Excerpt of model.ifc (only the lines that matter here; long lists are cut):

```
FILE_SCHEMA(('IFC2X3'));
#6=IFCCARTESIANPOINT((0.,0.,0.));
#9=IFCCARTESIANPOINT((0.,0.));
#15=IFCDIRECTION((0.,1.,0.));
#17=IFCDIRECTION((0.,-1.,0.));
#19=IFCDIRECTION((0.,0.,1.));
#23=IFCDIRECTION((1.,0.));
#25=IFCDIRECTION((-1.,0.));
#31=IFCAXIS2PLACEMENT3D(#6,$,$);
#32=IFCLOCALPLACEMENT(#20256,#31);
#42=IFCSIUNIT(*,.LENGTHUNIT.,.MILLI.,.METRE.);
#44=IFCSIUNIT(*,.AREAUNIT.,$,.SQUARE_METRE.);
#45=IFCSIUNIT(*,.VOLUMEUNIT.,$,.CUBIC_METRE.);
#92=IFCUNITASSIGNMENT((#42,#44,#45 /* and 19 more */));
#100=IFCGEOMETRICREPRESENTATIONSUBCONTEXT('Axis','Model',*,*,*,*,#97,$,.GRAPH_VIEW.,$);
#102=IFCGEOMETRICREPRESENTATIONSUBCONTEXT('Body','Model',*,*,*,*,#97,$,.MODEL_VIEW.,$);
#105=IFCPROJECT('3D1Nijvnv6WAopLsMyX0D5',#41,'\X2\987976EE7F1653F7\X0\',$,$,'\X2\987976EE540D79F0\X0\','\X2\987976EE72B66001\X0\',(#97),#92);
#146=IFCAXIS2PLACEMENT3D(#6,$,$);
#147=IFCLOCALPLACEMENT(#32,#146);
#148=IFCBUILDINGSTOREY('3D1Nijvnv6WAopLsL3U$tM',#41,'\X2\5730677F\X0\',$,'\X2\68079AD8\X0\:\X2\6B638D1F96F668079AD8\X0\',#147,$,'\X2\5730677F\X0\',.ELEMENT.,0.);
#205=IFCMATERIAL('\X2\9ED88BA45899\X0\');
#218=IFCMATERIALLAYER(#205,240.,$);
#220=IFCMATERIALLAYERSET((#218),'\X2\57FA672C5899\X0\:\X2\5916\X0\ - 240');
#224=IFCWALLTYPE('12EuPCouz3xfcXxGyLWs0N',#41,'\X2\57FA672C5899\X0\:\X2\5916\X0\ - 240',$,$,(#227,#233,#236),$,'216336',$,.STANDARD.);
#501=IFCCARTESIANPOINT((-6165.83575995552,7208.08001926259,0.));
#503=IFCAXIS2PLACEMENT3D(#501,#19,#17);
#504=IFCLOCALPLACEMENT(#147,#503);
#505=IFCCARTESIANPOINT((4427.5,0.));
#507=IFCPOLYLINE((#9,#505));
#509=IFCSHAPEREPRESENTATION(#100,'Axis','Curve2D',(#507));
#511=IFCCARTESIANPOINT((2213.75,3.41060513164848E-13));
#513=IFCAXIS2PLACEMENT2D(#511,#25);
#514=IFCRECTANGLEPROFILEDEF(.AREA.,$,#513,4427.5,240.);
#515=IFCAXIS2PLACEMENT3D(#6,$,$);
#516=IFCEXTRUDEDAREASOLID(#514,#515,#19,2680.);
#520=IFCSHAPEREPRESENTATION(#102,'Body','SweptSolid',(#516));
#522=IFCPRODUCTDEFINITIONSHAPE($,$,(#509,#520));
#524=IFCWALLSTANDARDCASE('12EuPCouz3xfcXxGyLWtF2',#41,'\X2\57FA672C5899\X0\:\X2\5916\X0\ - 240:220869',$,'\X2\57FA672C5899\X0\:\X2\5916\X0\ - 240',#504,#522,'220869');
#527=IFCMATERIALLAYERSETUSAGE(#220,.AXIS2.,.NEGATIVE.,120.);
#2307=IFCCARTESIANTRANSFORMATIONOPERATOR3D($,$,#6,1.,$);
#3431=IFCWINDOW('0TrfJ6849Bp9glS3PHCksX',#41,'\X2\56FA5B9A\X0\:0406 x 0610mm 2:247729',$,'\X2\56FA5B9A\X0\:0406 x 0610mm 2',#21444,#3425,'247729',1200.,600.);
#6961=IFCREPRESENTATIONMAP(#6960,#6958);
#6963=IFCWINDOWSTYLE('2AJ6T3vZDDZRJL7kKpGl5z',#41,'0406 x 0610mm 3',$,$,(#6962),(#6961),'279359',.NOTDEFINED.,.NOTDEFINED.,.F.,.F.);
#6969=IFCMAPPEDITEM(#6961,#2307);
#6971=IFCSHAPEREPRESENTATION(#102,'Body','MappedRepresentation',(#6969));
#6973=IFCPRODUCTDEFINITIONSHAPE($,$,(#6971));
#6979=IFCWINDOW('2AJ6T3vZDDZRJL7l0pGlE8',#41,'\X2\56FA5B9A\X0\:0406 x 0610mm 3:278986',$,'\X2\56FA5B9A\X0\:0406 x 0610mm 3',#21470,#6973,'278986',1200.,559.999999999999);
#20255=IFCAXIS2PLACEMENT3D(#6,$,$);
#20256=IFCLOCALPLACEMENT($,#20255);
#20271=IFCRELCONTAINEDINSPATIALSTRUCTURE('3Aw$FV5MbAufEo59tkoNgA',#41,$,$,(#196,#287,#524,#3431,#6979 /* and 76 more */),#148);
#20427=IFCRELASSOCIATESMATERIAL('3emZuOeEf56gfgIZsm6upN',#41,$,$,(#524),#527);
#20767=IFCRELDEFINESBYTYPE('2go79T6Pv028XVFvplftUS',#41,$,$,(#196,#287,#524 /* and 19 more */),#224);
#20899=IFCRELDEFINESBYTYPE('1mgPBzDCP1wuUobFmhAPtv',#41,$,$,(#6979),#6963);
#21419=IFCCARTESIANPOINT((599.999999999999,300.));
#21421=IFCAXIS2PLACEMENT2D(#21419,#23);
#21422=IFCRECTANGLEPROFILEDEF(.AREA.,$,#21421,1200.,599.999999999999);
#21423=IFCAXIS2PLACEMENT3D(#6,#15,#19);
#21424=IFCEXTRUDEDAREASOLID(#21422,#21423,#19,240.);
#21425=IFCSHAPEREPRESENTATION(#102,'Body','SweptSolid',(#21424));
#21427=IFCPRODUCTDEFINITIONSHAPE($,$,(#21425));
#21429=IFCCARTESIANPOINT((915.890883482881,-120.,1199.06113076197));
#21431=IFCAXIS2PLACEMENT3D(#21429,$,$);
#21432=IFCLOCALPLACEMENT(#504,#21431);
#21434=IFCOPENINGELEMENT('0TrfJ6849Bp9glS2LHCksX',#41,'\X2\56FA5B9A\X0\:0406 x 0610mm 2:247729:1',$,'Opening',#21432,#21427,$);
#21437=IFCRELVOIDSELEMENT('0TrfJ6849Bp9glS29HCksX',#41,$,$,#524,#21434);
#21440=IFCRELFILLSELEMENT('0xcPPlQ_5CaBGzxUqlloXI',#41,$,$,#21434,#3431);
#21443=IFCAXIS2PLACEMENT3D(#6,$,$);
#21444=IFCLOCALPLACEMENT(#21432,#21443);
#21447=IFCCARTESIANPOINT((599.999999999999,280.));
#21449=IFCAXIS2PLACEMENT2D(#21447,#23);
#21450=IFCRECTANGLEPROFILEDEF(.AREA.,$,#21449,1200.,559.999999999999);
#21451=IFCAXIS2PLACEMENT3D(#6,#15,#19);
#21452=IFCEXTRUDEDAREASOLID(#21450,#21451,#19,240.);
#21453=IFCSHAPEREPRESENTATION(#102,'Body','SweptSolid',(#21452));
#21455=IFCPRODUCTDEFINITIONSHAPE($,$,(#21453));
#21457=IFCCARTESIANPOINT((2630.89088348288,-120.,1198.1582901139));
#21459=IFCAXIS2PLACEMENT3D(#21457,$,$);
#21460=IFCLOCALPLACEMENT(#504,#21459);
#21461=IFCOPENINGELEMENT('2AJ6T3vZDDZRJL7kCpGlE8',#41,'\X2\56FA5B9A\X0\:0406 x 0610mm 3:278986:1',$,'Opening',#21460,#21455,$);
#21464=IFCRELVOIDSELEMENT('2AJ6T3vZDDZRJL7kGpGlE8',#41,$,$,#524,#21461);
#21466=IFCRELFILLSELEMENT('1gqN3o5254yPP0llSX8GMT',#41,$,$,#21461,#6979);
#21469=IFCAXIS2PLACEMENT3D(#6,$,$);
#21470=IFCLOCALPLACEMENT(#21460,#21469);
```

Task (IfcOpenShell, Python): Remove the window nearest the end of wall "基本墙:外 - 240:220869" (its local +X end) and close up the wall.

```python
import ifcopenshell
import ifcopenshell.api.feature
import ifcopenshell.api.root
import ifcopenshell.geom
import ifcopenshell.util.shape

model = ifcopenshell.open("model.ifc")
settings = ifcopenshell.geom.settings()


def volume(element):
    """Net volume in cubic metres, openings subtracted."""
    shape = ifcopenshell.geom.create_shape(settings, element)
    return ifcopenshell.util.shape.get_volume(shape.geometry)


window = model.by_guid("2AJ6T3vZDDZRJL7l0pGlE8")
opening = window.FillsVoids[0].RelatingOpeningElement
wall = opening.VoidsElements[0].RelatingBuildingElement
before = volume(wall)

ifcopenshell.api.root.remove_product(model, product=window)
ifcopenshell.api.feature.remove_feature(model, feature=opening)

after = volume(wall)

print(f"wall volume {before:.3f} -> {after:.3f} m3")

model.write("model_updated.ifc")
```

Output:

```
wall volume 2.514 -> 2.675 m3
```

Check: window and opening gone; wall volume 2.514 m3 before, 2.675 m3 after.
